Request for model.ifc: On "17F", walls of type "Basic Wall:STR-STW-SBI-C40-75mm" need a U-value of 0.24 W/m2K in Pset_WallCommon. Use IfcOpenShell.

First a look at what the model holds.

```python
import ifcopenshell
import ifcopenshell.util.element

model = ifcopenshell.open("model.ifc")
print(model.schema)
storey = next(s for s in model.by_type("IfcBuildingStorey") if s.Name == "17F")
walls = [e for e in ifcopenshell.util.element.get_decomposition(storey) if e.is_a("IfcWall")]
seen = {}
for e in walls:
    element_type = ifcopenshell.util.element.get_type(e)
    key = (element_type.Name if element_type != e and element_type else None, ifcopenshell.util.element.get_pset(e, "Pset_WallCommon", "ThermalTransmittance"))
    seen[key] = seen.get(key, 0) + 1
for (name, value), count in sorted(seen.items(), key=str):
    print(count, "x", name, "|", value)
```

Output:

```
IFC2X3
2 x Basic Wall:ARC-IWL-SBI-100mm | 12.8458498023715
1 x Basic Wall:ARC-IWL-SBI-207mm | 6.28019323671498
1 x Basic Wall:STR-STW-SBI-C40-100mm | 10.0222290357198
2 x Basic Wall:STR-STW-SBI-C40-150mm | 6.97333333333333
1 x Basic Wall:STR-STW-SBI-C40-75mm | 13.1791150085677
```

```python
import ifcopenshell
import ifcopenshell.api.pset
import ifcopenshell.util.element

model = ifcopenshell.open("model.ifc")

storey = next(s for s in model.by_type("IfcBuildingStorey") if s.Name == "17F")
walls = [e for e in ifcopenshell.util.element.get_decomposition(storey) if e.is_a("IfcWall")]

count = 0
for e in walls:
    element_type = ifcopenshell.util.element.get_type(e)
    if element_type in (None, e) or element_type.Name != "Basic Wall:STR-STW-SBI-C40-75mm":
        continue
    # add_pset returns the element's existing set when there is one.
    pset = ifcopenshell.api.pset.add_pset(model, product=e, name="Pset_WallCommon")
    ifcopenshell.api.pset.edit_pset(model, pset=pset, properties={"ThermalTransmittance": 0.24})
    count += 1

print(count, "walls updated")

model.write("model_rev.ifc")
```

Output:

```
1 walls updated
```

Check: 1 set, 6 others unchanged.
